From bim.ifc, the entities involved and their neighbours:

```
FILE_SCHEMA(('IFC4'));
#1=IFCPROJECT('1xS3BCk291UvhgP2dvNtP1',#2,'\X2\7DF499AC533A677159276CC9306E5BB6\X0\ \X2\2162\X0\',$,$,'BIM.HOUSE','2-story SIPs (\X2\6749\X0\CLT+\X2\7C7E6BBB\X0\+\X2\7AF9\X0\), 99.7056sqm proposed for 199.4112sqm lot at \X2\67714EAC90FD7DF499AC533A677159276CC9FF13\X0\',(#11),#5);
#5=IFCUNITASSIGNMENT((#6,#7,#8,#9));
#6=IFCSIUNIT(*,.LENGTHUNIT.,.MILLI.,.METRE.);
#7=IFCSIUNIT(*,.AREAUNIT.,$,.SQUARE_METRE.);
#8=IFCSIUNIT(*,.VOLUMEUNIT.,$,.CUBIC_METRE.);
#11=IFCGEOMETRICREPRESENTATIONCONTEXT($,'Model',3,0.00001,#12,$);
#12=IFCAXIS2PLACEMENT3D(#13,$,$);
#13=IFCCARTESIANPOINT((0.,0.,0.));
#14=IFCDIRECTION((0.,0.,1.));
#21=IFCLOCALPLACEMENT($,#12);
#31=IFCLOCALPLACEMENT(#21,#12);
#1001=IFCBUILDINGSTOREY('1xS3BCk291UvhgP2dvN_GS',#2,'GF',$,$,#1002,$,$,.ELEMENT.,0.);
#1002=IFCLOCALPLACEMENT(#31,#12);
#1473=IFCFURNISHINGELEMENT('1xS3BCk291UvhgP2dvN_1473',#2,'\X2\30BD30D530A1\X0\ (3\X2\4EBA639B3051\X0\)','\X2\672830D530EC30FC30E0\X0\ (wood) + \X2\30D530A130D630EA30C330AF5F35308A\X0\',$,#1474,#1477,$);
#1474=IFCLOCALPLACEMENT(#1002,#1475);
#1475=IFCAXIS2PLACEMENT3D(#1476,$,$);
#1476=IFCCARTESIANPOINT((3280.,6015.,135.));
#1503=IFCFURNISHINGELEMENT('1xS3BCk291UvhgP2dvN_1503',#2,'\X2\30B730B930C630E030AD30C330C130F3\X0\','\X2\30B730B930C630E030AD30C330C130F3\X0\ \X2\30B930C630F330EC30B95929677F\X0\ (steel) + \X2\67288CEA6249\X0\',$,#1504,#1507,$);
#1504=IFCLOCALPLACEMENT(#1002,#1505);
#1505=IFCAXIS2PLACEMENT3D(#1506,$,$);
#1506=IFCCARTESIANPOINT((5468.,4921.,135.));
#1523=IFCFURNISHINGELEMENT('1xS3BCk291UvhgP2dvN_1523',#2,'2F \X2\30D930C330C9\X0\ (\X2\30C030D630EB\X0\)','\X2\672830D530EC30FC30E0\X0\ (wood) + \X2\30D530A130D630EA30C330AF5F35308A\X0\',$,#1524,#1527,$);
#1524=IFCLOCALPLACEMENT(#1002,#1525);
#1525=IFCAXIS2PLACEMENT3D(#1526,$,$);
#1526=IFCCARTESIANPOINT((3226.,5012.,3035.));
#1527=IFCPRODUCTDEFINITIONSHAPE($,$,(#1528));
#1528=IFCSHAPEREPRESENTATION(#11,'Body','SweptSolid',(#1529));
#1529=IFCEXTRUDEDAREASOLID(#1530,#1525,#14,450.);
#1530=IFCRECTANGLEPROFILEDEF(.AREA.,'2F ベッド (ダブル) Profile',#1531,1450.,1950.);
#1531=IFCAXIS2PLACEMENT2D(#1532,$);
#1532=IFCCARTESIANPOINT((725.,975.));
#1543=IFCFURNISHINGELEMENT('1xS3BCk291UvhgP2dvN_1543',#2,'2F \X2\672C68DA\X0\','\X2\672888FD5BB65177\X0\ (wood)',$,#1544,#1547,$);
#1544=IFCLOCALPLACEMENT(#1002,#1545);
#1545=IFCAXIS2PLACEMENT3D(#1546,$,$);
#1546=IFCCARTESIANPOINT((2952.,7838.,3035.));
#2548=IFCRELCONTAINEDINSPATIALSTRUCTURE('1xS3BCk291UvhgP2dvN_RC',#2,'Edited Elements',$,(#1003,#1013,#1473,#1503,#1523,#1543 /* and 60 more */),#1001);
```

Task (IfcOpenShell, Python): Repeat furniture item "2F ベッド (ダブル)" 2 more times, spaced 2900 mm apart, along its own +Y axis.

```python
import ifcopenshell
import ifcopenshell.api.geometry
import ifcopenshell.api.root
import ifcopenshell.util.element
import ifcopenshell.util.placement
import ifcopenshell.util.unit

model = ifcopenshell.open("bim.ifc")
unit_scale = ifcopenshell.util.unit.calculate_unit_scale(model)


def reuse_history(source, copy):
    """copy_class also copies each property set's owner history, people and application; keep the originals."""
    for rel in copy.IsDefinedBy:
        if rel.is_a("IfcRelDefinesByProperties") and (history := rel.RelatingPropertyDefinition.OwnerHistory):
            rel.RelatingPropertyDefinition.OwnerHistory = source.OwnerHistory
            ifcopenshell.util.element.remove_deep2(model, history)


source = model.by_guid("1xS3BCk291UvhgP2dvN_1523")
base = ifcopenshell.util.placement.get_local_placement(source.ObjectPlacement)
step = base[:3, 1] * 2.9 / unit_scale

for i in range(1, 3):
    copy = ifcopenshell.api.root.copy_class(model, product=source)
    copy.Representation = ifcopenshell.util.element.copy_deep(
        model, source.Representation, exclude=["IfcGeometricRepresentationContext", "IfcRepresentationMap"]
    )
    reuse_history(source, copy)
    matrix = base.copy()
    matrix[:3, 3] += i * step
    print("added at", matrix[:3, 3].round(3) + 0.0)
    ifcopenshell.api.geometry.edit_object_placement(model, product=copy, matrix=matrix, is_si=False)

model.write("bim-out.ifc")
```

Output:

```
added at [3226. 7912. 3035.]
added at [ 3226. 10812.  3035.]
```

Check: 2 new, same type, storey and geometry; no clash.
